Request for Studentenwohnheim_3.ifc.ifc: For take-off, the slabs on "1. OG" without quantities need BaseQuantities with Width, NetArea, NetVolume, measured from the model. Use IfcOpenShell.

First a look at what the model holds.

```python
import ifcopenshell
import ifcopenshell.util.element
import ifcopenshell.util.unit

model = ifcopenshell.open("Studentenwohnheim_3.ifc.ifc")
print(model.schema)
for unit_type in ("LENGTHUNIT", "AREAUNIT", "VOLUMEUNIT"):
    print(unit_type, ifcopenshell.util.unit.calculate_unit_scale(model, unit_type))
storey = next(s for s in model.by_type("IfcBuildingStorey") if s.Name == "1. OG")
slabs = [e for e in ifcopenshell.util.element.get_decomposition(storey) if e.is_a("IfcSlab")]
for e in sorted(slabs, key=lambda e: e.id()):
    print(e.id(), e.is_a(), e.Name, list(ifcopenshell.util.element.get_psets(e, qtos_only=True)), sep=" | ")
```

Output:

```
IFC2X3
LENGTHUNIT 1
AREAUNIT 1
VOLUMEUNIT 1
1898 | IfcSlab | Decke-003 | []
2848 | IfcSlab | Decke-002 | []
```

```python
import ifcopenshell
import ifcopenshell.api.pset
import ifcopenshell.geom
import ifcopenshell.util.element
import ifcopenshell.util.shape
import ifcopenshell.util.unit

model = ifcopenshell.open("Studentenwohnheim_3.ifc.ifc")
unit_scale = ifcopenshell.util.unit.calculate_unit_scale(model)
area_scale = ifcopenshell.util.unit.calculate_unit_scale(model, "AREAUNIT")
volume_scale = ifcopenshell.util.unit.calculate_unit_scale(model, "VOLUMEUNIT")
settings = ifcopenshell.geom.settings()

storey = next(s for s in model.by_type("IfcBuildingStorey") if s.Name == "1. OG")
slabs = [e for e in ifcopenshell.util.element.get_decomposition(storey) if e.is_a("IfcSlab")]

for e in sorted(slabs, key=lambda e: e.id()):
    if ifcopenshell.util.element.get_psets(e, qtos_only=True, should_inherit=False):
        continue
    # Geometry comes back in metres, in the element's own axes.
    shape = ifcopenshell.geom.create_shape(settings, e)
    values = {
        "Width": ifcopenshell.util.shape.get_z(shape.geometry) / unit_scale,
        "NetArea": ifcopenshell.util.shape.get_footprint_area(shape.geometry) / area_scale,
        "NetVolume": ifcopenshell.util.shape.get_volume(shape.geometry) / volume_scale,
    }
    qto = ifcopenshell.api.pset.add_qto(model, product=e, name="BaseQuantities")
    ifcopenshell.api.pset.edit_qto(model, qto=qto, properties=values)
    print(e.id(), {k: round(v, 3) for k, v in values.items()})

model.write("Studentenwohnheim_3.ifc_v2.ifc")
```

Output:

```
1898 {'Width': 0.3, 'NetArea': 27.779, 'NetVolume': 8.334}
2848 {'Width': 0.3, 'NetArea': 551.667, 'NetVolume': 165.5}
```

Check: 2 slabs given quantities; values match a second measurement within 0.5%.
